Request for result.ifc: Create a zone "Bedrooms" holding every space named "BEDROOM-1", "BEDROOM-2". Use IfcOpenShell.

First a look at what the model holds.

```python
import ifcopenshell

model = ifcopenshell.open("result.ifc")
print(model.schema)
seen = {}
for space in model.by_type("IfcSpace"):
    seen[space.Name] = seen.get(space.Name, 0) + 1
for name, count in sorted(seen.items(), key=str):
    print(count, "x", name)
print("zones:", [z.Name for z in model.by_type("IfcZone")][:20])
```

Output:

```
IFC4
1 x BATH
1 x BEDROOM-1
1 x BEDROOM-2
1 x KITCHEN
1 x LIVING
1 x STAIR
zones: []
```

```python
import ifcopenshell
import ifcopenshell.api.group
import ifcopenshell.api.root

model = ifcopenshell.open("result.ifc")

names = {"BEDROOM-1", "BEDROOM-2"}
spaces = [s for s in model.by_type("IfcSpace") if s.Name in names]

zone = ifcopenshell.api.root.create_entity(model, ifc_class="IfcZone", name="Bedrooms")
ifcopenshell.api.group.assign_group(model, products=spaces, group=zone)
print(len(spaces), "spaces in", zone.Name)

model.write("result_updated.ifc")
```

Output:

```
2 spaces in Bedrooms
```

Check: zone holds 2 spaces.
